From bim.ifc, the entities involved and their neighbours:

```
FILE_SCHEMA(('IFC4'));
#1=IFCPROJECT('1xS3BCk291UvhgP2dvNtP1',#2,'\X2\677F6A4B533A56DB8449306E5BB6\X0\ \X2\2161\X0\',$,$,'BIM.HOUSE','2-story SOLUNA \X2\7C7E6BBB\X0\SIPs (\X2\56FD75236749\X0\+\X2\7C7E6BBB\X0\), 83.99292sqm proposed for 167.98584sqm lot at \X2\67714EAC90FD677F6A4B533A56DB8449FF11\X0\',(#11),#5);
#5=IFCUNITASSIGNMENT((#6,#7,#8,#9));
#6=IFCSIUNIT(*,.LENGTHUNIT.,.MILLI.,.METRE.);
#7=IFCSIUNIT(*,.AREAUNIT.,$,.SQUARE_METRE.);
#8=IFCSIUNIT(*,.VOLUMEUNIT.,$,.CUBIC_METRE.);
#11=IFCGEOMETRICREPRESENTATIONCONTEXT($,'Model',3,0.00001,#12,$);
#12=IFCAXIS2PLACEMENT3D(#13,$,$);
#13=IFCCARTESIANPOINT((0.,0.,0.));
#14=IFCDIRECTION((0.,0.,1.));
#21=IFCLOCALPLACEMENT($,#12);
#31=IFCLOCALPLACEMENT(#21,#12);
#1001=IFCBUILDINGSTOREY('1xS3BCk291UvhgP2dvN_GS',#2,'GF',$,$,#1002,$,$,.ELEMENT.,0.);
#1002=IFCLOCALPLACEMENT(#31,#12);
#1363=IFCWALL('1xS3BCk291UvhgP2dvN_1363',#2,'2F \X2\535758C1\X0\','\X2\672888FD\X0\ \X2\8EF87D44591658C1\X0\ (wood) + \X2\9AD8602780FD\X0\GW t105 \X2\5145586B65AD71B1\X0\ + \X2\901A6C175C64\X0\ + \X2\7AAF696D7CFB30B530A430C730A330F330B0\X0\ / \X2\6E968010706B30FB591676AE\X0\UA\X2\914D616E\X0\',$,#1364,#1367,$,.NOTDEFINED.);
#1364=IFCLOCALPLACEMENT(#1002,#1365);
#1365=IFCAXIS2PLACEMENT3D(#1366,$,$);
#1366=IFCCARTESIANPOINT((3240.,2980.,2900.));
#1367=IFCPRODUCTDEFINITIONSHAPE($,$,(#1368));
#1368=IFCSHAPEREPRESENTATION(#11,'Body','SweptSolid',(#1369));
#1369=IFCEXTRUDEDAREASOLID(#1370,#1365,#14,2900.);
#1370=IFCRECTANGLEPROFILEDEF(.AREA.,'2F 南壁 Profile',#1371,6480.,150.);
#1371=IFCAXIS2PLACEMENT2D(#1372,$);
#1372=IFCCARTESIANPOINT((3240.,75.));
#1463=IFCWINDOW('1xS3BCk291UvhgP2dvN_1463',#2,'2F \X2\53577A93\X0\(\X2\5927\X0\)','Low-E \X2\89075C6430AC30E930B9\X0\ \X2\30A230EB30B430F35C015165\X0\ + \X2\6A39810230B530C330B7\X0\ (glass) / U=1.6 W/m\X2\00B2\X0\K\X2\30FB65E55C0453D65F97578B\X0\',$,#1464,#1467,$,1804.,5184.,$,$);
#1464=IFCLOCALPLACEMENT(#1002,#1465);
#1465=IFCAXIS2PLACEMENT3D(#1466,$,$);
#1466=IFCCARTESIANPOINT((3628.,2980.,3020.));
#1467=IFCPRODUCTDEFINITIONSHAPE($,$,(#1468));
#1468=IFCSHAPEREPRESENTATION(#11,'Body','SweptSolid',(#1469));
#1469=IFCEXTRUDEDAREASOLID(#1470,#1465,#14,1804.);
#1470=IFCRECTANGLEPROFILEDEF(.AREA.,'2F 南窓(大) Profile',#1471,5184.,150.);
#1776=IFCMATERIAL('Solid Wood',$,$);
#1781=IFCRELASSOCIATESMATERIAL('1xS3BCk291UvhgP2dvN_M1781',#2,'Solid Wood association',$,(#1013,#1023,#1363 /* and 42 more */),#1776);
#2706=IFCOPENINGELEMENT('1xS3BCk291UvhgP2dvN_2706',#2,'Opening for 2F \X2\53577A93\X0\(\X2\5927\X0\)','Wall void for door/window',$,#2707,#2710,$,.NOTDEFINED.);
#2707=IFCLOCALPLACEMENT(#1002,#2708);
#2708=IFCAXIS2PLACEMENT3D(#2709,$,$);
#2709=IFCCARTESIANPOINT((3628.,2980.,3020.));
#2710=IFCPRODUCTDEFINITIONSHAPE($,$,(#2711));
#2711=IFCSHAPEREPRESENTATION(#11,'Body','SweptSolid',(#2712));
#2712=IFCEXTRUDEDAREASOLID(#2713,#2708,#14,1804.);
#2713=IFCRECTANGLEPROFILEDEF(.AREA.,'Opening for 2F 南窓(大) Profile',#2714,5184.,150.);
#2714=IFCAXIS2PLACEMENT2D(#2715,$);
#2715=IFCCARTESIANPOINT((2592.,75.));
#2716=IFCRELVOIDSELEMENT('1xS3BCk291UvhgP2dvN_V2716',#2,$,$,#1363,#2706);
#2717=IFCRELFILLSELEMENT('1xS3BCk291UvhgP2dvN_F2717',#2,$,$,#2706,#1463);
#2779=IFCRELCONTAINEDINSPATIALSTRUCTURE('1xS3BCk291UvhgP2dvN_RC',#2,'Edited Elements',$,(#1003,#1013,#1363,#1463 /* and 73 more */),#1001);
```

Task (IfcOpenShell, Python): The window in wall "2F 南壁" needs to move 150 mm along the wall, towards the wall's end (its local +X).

```python
import ifcopenshell
import ifcopenshell.api.geometry
import ifcopenshell.util.placement
import ifcopenshell.util.unit

model = ifcopenshell.open("bim.ifc")
unit_scale = ifcopenshell.util.unit.calculate_unit_scale(model)

window = model.by_guid("1xS3BCk291UvhgP2dvN_1463")
opening = window.FillsVoids[0].RelatingOpeningElement
wall = opening.VoidsElements[0].RelatingBuildingElement

wall_matrix = ifcopenshell.util.placement.get_local_placement(wall.ObjectPlacement)
shift = wall_matrix[:3, 0] * 0.15 / unit_scale
before = ifcopenshell.util.placement.get_local_placement(window.ObjectPlacement)[:3, 3].copy()

# The window is not placed relative to its opening, so move both.
for product in (opening, window):
    matrix = ifcopenshell.util.placement.get_local_placement(product.ObjectPlacement)
    matrix[:3, 3] += shift
    ifcopenshell.api.geometry.edit_object_placement(model, product=product, matrix=matrix, is_si=False)

after = ifcopenshell.util.placement.get_local_placement(window.ObjectPlacement)[:3, 3]
print("window moved by", (after - before).round(3) + 0.0)

model.write("bim_v2.ifc")
```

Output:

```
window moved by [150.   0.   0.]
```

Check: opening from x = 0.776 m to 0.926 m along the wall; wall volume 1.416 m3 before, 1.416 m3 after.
